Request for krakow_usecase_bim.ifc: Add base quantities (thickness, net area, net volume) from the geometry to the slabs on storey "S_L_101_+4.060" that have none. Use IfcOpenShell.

First a look at what the model holds.

```python
import ifcopenshell
import ifcopenshell.util.element
import ifcopenshell.util.unit

model = ifcopenshell.open("krakow_usecase_bim.ifc")
print(model.schema)
for unit_type in ("LENGTHUNIT", "AREAUNIT", "VOLUMEUNIT"):
    print(unit_type, ifcopenshell.util.unit.calculate_unit_scale(model, unit_type))
storey = next(s for s in model.by_type("IfcBuildingStorey") if s.Name == "S_L_101_+4.060")
slabs = [e for e in ifcopenshell.util.element.get_decomposition(storey) if e.is_a("IfcSlab")]
for e in sorted(slabs, key=lambda e: e.id()):
    print(e.id(), e.is_a(), e.Name, list(ifcopenshell.util.element.get_psets(e, qtos_only=True)), sep=" | ")
```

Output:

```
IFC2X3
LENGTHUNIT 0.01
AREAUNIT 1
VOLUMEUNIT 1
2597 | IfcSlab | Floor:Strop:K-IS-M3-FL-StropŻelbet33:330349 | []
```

```python
import ifcopenshell
import ifcopenshell.api.pset
import ifcopenshell.geom
import ifcopenshell.util.element
import ifcopenshell.util.shape
import ifcopenshell.util.unit

model = ifcopenshell.open("krakow_usecase_bim.ifc")
unit_scale = ifcopenshell.util.unit.calculate_unit_scale(model)
area_scale = ifcopenshell.util.unit.calculate_unit_scale(model, "AREAUNIT")
volume_scale = ifcopenshell.util.unit.calculate_unit_scale(model, "VOLUMEUNIT")
settings = ifcopenshell.geom.settings()

storey = next(s for s in model.by_type("IfcBuildingStorey") if s.Name == "S_L_101_+4.060")
slabs = [e for e in ifcopenshell.util.element.get_decomposition(storey) if e.is_a("IfcSlab")]

for e in sorted(slabs, key=lambda e: e.id()):
    if ifcopenshell.util.element.get_psets(e, qtos_only=True, should_inherit=False):
        continue
    # Geometry comes back in metres, in the element's own axes.
    shape = ifcopenshell.geom.create_shape(settings, e)
    values = {
        "Width": ifcopenshell.util.shape.get_z(shape.geometry) / unit_scale,
        "NetArea": ifcopenshell.util.shape.get_footprint_area(shape.geometry) / area_scale,
        "NetVolume": ifcopenshell.util.shape.get_volume(shape.geometry) / volume_scale,
    }
    qto = ifcopenshell.api.pset.add_qto(model, product=e, name="BaseQuantities")
    ifcopenshell.api.pset.edit_qto(model, qto=qto, properties=values)
    print(e.id(), {k: round(v, 3) for k, v in values.items()})

model.write("krakow_usecase_bim-out.ifc")
```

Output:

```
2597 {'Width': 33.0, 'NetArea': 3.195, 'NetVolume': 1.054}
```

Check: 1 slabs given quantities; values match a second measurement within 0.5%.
